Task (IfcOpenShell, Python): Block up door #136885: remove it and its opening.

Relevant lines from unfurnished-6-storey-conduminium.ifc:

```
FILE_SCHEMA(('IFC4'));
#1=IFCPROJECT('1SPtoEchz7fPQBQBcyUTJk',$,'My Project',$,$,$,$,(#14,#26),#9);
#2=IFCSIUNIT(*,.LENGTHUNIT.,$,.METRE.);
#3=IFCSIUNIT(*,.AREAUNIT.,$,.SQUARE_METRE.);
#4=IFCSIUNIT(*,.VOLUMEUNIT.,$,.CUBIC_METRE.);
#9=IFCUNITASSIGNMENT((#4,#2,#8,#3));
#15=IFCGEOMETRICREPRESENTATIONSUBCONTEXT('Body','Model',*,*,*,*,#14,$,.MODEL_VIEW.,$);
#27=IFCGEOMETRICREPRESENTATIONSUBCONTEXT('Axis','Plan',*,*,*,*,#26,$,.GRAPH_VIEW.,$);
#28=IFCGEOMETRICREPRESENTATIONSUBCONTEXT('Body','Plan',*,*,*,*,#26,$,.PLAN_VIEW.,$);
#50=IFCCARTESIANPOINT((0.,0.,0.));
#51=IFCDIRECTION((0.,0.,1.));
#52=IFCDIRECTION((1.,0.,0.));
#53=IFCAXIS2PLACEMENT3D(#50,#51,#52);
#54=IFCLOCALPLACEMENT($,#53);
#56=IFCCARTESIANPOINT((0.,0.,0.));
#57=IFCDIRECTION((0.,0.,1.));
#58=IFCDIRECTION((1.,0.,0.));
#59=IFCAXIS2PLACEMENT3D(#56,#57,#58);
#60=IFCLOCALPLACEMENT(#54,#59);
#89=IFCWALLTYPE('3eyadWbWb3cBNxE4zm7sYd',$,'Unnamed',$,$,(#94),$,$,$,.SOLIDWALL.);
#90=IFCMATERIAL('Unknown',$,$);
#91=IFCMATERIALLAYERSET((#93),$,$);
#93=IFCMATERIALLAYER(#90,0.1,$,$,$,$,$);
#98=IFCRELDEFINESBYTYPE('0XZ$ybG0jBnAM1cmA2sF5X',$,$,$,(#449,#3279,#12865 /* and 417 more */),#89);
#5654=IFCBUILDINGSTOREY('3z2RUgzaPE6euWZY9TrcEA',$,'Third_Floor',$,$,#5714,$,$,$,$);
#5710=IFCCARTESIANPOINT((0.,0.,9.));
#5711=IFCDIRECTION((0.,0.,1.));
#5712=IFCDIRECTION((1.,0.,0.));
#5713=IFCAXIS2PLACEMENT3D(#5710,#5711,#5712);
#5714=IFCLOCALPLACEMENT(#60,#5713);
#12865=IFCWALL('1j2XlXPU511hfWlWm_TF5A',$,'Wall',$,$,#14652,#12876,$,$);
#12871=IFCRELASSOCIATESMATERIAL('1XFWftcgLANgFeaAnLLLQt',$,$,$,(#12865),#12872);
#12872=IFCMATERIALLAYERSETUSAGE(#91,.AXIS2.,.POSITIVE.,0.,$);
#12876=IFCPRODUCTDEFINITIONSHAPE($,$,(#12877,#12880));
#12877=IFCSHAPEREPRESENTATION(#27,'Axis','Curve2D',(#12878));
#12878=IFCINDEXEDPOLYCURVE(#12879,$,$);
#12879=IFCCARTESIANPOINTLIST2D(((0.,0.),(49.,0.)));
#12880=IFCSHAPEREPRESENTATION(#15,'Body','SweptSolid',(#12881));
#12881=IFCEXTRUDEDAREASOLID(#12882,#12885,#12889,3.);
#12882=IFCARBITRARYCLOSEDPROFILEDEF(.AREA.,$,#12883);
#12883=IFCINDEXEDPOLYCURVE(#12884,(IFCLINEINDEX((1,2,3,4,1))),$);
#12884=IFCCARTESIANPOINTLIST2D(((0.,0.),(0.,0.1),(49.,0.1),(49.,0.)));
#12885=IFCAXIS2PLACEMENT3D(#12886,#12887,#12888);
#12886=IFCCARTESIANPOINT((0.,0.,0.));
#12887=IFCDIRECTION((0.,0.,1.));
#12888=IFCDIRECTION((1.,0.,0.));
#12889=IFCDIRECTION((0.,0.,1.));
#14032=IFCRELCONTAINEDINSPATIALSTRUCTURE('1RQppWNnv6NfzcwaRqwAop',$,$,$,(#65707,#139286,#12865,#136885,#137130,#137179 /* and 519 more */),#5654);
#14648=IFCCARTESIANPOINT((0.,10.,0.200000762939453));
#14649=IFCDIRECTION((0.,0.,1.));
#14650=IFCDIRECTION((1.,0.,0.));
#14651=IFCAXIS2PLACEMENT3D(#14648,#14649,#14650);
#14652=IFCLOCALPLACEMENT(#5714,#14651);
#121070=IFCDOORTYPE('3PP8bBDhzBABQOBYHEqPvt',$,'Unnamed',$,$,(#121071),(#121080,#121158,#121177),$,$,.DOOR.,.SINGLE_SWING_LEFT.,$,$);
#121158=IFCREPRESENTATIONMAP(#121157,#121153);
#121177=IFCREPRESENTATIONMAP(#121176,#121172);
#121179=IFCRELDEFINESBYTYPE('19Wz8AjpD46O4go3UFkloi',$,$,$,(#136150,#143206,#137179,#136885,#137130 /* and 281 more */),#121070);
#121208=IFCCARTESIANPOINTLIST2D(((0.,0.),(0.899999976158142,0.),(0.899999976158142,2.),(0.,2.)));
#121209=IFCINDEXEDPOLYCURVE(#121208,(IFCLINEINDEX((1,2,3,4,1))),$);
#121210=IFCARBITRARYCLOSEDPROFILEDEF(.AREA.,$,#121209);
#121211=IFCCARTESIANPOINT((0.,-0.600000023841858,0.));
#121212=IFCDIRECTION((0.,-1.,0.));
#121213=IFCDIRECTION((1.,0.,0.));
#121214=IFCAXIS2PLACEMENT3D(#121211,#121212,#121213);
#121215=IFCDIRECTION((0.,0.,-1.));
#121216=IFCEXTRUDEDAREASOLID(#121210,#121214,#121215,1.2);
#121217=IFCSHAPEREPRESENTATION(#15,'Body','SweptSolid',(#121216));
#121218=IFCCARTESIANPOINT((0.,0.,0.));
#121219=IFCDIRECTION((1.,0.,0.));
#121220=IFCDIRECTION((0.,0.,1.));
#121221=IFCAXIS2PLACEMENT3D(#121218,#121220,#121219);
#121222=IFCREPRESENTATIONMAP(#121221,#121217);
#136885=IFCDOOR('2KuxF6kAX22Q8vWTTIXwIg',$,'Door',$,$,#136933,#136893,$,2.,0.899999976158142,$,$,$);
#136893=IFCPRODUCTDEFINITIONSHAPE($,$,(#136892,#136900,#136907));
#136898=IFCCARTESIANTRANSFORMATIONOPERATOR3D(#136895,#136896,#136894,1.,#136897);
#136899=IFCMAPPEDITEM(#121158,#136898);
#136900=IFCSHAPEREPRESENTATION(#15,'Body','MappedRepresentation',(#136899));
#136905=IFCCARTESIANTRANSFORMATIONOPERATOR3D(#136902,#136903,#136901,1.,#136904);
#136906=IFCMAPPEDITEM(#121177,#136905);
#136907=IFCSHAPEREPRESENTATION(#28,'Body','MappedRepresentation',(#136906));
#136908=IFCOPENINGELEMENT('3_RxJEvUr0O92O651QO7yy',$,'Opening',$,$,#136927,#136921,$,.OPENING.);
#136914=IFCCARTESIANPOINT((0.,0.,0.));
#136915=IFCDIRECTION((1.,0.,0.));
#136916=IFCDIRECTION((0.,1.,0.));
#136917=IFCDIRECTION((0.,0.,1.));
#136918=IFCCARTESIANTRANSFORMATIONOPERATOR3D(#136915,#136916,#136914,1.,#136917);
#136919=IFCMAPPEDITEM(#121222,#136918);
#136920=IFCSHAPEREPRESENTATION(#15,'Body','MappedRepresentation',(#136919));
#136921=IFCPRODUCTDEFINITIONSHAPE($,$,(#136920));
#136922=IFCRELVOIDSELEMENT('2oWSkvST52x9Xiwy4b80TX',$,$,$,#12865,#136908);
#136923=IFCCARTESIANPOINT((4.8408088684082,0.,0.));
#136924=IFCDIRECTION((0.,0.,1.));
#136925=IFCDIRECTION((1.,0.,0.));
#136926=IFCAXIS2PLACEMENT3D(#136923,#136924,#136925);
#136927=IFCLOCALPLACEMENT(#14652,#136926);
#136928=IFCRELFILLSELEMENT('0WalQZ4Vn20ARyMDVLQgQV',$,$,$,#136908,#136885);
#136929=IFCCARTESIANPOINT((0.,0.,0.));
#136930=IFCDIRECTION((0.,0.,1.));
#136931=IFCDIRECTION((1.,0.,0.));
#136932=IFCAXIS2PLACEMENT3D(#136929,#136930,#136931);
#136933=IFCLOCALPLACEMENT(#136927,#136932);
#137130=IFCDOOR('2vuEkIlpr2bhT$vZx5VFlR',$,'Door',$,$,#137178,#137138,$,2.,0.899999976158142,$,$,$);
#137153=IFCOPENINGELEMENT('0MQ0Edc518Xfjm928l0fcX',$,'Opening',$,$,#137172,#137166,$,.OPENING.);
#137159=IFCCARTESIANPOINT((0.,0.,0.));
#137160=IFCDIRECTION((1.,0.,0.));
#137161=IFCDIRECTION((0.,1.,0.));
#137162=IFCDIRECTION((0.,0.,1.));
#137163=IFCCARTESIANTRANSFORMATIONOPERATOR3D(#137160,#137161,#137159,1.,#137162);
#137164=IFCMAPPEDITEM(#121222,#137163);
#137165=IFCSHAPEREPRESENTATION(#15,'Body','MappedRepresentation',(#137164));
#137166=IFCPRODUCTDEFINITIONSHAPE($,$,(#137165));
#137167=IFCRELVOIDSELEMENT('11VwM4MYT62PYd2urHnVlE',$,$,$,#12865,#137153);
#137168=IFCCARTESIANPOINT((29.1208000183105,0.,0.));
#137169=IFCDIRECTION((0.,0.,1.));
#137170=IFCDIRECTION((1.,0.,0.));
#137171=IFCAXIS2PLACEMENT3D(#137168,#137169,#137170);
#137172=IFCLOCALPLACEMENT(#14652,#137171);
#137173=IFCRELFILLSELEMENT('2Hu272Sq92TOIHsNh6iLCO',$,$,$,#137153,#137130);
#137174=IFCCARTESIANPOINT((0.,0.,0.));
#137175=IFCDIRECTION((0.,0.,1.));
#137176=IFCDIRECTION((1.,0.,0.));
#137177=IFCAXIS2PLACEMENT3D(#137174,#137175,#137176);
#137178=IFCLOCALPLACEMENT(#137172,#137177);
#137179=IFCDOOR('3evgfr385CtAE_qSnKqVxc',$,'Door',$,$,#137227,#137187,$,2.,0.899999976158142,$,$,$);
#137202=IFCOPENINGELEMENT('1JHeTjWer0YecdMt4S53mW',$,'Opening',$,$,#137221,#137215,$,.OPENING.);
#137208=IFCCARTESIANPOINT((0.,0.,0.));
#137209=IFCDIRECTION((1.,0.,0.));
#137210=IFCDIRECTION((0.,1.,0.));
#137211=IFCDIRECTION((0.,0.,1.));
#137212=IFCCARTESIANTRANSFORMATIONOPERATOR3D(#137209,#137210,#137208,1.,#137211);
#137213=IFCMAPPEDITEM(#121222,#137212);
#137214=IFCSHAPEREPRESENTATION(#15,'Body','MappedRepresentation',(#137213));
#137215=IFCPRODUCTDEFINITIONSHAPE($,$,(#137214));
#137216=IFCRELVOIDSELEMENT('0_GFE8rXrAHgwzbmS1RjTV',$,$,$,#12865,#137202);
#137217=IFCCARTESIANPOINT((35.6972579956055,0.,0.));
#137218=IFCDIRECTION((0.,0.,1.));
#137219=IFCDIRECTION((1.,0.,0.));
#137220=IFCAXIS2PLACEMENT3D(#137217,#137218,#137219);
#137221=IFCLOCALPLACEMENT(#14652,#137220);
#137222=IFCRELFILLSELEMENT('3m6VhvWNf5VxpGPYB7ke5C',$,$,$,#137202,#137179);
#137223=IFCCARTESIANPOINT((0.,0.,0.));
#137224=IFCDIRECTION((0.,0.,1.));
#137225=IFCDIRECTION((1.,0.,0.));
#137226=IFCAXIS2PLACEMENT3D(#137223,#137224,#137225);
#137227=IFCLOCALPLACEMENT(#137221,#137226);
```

```python
import ifcopenshell
import ifcopenshell.api.feature
import ifcopenshell.api.root
import ifcopenshell.geom
import ifcopenshell.util.shape

model = ifcopenshell.open("unfurnished-6-storey-conduminium.ifc")
settings = ifcopenshell.geom.settings()


def volume(element):
    """Net volume in cubic metres, openings subtracted."""
    shape = ifcopenshell.geom.create_shape(settings, element)
    return ifcopenshell.util.shape.get_volume(shape.geometry)


door = model.by_id(136885)
opening = door.FillsVoids[0].RelatingOpeningElement
wall = opening.VoidsElements[0].RelatingBuildingElement
before = volume(wall)

ifcopenshell.api.root.remove_product(model, product=door)
ifcopenshell.api.feature.remove_feature(model, feature=opening)

after = volume(wall)

print(f"wall volume {before:.3f} -> {after:.3f} m3")

model.write("unfurnished-6-storey-conduminium_edited.ifc")
```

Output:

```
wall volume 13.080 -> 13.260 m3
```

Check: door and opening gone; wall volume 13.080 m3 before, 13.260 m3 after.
